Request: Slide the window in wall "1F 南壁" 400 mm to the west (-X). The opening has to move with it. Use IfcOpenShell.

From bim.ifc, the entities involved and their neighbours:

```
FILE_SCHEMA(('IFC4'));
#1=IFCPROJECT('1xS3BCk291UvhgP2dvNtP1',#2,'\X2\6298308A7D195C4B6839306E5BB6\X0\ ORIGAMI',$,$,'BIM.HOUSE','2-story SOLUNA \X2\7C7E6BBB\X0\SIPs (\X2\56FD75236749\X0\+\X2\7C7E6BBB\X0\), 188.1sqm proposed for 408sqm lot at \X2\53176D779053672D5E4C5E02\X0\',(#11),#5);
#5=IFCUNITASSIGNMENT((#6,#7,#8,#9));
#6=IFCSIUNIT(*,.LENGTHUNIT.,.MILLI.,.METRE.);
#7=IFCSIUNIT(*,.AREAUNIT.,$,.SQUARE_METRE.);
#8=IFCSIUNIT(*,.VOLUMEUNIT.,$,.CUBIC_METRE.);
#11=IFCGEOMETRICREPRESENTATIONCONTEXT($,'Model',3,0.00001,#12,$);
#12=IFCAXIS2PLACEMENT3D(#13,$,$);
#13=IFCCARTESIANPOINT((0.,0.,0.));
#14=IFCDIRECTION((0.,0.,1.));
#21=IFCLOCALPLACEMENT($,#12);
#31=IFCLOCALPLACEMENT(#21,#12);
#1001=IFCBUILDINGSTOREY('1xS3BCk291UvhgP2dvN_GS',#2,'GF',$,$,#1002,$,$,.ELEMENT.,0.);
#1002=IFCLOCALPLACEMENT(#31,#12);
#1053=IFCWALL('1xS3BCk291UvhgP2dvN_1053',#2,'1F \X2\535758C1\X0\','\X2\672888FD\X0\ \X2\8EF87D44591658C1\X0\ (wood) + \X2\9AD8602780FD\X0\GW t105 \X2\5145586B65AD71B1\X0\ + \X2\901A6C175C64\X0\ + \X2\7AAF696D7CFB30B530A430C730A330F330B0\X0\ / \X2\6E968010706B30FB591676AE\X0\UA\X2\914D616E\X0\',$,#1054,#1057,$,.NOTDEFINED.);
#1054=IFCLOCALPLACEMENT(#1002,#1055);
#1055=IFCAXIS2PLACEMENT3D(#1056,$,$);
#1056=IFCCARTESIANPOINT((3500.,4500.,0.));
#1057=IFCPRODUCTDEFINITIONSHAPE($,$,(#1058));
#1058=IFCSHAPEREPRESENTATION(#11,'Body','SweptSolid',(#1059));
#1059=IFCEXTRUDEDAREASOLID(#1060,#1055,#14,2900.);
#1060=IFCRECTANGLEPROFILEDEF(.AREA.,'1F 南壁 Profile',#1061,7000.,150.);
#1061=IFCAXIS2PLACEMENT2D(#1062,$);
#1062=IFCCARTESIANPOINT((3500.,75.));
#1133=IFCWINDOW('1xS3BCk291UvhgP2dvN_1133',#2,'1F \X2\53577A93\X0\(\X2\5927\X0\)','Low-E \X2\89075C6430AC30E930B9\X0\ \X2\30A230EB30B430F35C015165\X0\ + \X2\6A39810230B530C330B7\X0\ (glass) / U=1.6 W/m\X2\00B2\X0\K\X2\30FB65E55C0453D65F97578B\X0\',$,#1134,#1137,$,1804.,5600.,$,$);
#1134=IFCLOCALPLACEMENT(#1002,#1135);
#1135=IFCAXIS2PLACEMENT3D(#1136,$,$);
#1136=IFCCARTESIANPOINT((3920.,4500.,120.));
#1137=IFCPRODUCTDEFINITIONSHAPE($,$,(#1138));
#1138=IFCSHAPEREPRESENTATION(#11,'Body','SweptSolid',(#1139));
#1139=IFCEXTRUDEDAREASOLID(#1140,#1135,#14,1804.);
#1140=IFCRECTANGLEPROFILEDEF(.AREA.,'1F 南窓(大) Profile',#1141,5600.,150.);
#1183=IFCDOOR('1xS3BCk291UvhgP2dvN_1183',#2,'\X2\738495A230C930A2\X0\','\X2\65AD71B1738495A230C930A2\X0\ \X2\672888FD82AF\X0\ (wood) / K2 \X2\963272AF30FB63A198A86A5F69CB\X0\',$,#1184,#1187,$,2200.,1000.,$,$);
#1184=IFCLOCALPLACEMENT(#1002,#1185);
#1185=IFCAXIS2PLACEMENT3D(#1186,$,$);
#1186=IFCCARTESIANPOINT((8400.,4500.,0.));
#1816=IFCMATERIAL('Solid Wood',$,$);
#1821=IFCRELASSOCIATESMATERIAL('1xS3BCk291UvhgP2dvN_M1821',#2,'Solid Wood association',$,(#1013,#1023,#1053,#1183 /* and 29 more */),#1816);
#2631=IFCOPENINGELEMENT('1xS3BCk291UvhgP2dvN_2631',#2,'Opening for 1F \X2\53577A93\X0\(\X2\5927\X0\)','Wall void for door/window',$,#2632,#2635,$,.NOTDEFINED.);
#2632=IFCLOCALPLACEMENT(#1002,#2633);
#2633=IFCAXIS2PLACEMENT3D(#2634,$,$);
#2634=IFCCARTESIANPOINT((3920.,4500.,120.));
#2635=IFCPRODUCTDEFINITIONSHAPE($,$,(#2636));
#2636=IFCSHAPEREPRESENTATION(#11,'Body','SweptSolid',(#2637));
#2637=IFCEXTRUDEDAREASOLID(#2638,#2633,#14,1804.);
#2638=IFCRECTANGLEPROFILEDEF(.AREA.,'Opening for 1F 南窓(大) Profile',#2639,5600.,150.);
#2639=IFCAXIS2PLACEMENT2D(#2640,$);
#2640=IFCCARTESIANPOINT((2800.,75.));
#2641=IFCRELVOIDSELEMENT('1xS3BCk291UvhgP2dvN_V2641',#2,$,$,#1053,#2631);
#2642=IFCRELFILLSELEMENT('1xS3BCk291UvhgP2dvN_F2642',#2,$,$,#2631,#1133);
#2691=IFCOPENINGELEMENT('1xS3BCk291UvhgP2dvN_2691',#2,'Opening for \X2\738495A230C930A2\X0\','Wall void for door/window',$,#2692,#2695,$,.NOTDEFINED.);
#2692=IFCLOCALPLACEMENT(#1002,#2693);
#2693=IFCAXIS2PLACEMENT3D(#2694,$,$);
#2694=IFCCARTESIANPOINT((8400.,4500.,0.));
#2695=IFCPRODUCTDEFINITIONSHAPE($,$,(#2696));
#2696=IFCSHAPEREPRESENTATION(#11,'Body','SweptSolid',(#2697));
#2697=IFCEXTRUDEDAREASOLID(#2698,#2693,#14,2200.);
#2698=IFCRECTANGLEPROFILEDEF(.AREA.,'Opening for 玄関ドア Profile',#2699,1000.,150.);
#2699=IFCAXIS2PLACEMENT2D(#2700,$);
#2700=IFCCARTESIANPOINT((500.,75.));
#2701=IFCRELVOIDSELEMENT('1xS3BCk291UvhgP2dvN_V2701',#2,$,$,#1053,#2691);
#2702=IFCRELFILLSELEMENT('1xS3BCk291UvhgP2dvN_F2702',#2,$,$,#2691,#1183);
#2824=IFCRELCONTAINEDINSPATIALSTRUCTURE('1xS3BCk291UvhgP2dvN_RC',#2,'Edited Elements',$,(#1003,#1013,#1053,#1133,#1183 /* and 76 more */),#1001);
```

```python
import ifcopenshell
import ifcopenshell.api.geometry
import ifcopenshell.util.placement

model = ifcopenshell.open("bim.ifc")

window = model.by_guid("1xS3BCk291UvhgP2dvN_1133")
opening = window.FillsVoids[0].RelatingOpeningElement
wall = opening.VoidsElements[0].RelatingBuildingElement

wall_matrix = ifcopenshell.util.placement.get_local_placement(wall.ObjectPlacement)
shift = wall_matrix[:3, 0] * -400.0
before = ifcopenshell.util.placement.get_local_placement(window.ObjectPlacement)[:3, 3].copy()

# The window is not placed relative to its opening, so move both.
for product in (opening, window):
    matrix = ifcopenshell.util.placement.get_local_placement(product.ObjectPlacement)
    matrix[:3, 3] += shift
    ifcopenshell.api.geometry.edit_object_placement(model, product=product, matrix=matrix, is_si=False)

after = ifcopenshell.util.placement.get_local_placement(window.ObjectPlacement)[:3, 3]
print("window moved by", (after - before).round(3) + 0.0)

model.write("bim_rev.ifc")
```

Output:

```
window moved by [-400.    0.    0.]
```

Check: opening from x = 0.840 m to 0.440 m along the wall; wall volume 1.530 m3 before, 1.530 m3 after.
